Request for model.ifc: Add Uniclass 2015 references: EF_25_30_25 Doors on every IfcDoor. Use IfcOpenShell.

First a look at what the model holds.

```python
import ifcopenshell

model = ifcopenshell.open("model.ifc")
print(model.schema)
print("classifications:", [c.Name for c in model.by_type("IfcClassification")])
for ifc_class in ("IfcDoor", "IfcRoof", "IfcStair", "IfcWall", "IfcWindow"):
    print(ifc_class, len(model.by_type(ifc_class)))
```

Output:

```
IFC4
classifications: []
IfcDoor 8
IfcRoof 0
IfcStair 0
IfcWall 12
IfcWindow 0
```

```python
import ifcopenshell
import ifcopenshell.api.classification

model = ifcopenshell.open("model.ifc")

system = ifcopenshell.api.classification.add_classification(model, classification="Uniclass 2015")

codes = {
    "IfcDoor": ("EF_25_30_25", "Doors"),
}
for ifc_class, (code, name) in codes.items():
    products = model.by_type(ifc_class)
    ifcopenshell.api.classification.add_reference(
        model, products=products, classification=system, identification=code, name=name
    )
    print(code, len(products))

model.write("model_updated.ifc")
```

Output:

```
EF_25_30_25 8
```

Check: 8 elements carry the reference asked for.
